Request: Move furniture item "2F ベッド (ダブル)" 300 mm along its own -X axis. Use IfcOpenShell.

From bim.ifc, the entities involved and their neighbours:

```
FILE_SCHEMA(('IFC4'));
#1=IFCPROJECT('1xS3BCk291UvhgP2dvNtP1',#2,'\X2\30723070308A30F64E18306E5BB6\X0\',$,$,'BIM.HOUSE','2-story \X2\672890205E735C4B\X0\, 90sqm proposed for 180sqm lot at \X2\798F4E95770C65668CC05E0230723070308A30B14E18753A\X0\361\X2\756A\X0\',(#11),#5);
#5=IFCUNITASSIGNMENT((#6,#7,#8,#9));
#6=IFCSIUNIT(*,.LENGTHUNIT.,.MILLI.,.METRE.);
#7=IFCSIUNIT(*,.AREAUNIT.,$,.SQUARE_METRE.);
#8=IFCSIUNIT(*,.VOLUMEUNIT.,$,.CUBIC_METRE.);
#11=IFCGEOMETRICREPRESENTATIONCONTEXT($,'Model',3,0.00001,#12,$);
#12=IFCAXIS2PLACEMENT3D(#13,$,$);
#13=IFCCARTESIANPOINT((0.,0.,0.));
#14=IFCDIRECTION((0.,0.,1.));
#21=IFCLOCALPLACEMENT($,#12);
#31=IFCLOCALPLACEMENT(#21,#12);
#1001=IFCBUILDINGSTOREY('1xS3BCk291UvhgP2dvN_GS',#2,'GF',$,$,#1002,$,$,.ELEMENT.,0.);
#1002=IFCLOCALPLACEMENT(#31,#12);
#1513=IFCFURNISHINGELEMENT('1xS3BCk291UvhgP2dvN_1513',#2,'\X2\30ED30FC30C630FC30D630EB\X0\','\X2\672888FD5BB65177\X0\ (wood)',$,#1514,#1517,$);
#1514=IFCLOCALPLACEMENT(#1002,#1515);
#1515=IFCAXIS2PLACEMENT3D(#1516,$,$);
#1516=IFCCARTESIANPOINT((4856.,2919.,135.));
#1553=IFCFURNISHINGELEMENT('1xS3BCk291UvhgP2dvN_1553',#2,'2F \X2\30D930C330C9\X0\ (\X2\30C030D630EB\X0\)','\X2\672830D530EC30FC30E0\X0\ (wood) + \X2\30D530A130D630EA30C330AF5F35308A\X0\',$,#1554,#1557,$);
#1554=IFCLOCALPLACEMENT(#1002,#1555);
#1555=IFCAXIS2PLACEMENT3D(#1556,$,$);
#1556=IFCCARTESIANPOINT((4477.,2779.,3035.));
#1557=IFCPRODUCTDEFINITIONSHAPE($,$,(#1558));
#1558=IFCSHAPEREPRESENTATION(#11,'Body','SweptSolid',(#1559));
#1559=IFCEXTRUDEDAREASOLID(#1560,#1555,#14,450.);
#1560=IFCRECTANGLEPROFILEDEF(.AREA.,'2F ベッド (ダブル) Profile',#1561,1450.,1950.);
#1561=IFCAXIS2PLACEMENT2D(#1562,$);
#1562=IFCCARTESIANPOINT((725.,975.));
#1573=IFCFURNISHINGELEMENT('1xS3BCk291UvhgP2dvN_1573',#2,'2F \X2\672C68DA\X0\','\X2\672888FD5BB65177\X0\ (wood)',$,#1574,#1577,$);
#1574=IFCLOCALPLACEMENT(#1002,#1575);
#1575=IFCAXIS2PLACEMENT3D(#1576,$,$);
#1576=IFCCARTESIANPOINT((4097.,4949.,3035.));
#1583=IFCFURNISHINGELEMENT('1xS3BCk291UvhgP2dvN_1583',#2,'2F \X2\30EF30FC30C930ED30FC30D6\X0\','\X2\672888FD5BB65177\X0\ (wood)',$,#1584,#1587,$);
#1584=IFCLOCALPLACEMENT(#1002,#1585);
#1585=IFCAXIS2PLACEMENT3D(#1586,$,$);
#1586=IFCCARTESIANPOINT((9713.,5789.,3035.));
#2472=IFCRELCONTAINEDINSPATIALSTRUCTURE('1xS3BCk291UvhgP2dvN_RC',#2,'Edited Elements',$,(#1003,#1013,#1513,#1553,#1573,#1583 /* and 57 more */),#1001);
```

```python
import ifcopenshell
import ifcopenshell.api.geometry
import ifcopenshell.util.placement

model = ifcopenshell.open("bim.ifc")

item = model.by_id(1553)
matrix = ifcopenshell.util.placement.get_local_placement(item.ObjectPlacement)
matrix[:3, 3] -= matrix[:3, 0] * 300.0
ifcopenshell.api.geometry.edit_object_placement(model, product=item, matrix=matrix, is_si=False)

print(ifcopenshell.util.placement.get_local_placement(item.ObjectPlacement).round(3) + 0.0)

model.write("bim_updated.ifc")
```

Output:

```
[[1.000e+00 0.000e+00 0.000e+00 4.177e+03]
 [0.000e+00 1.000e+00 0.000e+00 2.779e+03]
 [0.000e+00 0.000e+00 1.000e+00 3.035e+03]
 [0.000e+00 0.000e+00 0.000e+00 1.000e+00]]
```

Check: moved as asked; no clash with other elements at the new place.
